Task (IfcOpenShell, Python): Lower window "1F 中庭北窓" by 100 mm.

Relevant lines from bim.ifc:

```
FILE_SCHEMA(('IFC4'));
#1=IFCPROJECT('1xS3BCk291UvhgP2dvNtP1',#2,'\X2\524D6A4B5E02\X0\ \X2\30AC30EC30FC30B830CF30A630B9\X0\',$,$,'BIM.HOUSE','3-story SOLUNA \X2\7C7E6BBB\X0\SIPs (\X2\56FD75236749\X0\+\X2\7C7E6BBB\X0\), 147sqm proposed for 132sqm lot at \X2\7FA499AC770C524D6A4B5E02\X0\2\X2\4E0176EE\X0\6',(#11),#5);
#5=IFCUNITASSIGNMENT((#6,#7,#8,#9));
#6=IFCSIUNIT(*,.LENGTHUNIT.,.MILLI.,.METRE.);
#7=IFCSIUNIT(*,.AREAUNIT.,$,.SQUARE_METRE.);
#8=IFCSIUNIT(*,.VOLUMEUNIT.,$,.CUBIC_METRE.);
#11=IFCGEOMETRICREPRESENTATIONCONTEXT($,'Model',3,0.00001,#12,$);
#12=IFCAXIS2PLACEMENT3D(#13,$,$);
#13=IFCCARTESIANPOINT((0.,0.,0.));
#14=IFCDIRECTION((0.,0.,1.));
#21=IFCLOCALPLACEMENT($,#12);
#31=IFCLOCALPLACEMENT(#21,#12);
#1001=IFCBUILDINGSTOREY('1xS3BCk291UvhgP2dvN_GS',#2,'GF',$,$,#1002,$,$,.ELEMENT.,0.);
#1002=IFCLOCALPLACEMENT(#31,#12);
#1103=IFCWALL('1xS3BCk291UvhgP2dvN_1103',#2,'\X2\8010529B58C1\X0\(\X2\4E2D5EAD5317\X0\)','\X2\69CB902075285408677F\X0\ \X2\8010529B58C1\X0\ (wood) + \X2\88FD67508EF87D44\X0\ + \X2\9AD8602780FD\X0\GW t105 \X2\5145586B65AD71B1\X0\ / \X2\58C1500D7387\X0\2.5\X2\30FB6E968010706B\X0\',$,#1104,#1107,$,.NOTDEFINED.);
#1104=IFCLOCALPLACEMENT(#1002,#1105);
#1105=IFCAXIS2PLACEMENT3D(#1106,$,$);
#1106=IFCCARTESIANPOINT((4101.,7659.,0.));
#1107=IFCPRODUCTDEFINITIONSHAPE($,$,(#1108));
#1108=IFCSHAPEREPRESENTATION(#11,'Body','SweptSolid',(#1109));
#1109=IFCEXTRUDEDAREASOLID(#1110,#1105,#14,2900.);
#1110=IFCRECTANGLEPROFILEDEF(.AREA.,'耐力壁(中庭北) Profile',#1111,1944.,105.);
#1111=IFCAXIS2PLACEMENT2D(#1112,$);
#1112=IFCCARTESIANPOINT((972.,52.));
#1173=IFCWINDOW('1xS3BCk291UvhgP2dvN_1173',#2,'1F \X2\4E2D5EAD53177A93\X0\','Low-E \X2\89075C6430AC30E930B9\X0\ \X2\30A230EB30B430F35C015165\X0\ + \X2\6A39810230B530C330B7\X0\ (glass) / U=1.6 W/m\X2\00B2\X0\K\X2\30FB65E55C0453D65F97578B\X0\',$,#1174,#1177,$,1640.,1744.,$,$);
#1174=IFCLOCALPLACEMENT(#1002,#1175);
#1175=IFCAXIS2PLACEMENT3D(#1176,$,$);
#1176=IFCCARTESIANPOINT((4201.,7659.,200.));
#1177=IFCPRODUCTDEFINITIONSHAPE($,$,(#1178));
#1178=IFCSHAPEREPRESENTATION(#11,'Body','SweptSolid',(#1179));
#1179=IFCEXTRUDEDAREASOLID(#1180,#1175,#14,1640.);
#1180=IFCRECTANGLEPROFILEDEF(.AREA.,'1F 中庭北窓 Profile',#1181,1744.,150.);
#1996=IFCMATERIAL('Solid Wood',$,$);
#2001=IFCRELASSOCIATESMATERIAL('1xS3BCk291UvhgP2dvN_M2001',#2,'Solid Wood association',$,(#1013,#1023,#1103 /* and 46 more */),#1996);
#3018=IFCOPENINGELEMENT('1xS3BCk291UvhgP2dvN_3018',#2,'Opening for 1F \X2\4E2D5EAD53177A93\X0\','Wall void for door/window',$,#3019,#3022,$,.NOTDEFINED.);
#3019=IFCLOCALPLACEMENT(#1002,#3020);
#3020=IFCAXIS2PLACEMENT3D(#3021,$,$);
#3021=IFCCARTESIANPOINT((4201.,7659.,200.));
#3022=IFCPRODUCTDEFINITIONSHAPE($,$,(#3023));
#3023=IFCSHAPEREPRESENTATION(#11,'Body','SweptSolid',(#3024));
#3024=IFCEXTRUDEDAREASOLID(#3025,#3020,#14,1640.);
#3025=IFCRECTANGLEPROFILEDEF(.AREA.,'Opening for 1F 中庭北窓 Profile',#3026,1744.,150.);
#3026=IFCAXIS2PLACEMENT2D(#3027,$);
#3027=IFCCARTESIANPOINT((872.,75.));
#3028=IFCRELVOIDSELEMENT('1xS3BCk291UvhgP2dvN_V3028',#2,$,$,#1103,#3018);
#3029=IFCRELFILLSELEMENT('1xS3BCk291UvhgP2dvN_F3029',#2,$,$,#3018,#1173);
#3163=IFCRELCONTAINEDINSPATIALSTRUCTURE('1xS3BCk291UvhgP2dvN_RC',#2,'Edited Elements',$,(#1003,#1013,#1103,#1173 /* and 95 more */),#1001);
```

```python
import numpy as np
import ifcopenshell
import ifcopenshell.api.geometry
import ifcopenshell.util.placement
import ifcopenshell.util.unit

model = ifcopenshell.open("bim.ifc")
unit_scale = ifcopenshell.util.unit.calculate_unit_scale(model)

window = model.by_guid("1xS3BCk291UvhgP2dvN_1173")
opening = window.FillsVoids[0].RelatingOpeningElement
dz = -0.1 / unit_scale

shift = np.array([0.0, 0.0, dz])
# The window is not placed relative to its opening, so move both.
for product in (opening, window):
    matrix = ifcopenshell.util.placement.get_local_placement(product.ObjectPlacement)
    matrix[:3, 3] += shift
    ifcopenshell.api.geometry.edit_object_placement(model, product=product, matrix=matrix, is_si=False)

print(f"moved by {dz * unit_scale:+.3f} m")

model.write("bim-out.ifc")
```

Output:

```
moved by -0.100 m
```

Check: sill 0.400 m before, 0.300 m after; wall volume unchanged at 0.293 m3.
